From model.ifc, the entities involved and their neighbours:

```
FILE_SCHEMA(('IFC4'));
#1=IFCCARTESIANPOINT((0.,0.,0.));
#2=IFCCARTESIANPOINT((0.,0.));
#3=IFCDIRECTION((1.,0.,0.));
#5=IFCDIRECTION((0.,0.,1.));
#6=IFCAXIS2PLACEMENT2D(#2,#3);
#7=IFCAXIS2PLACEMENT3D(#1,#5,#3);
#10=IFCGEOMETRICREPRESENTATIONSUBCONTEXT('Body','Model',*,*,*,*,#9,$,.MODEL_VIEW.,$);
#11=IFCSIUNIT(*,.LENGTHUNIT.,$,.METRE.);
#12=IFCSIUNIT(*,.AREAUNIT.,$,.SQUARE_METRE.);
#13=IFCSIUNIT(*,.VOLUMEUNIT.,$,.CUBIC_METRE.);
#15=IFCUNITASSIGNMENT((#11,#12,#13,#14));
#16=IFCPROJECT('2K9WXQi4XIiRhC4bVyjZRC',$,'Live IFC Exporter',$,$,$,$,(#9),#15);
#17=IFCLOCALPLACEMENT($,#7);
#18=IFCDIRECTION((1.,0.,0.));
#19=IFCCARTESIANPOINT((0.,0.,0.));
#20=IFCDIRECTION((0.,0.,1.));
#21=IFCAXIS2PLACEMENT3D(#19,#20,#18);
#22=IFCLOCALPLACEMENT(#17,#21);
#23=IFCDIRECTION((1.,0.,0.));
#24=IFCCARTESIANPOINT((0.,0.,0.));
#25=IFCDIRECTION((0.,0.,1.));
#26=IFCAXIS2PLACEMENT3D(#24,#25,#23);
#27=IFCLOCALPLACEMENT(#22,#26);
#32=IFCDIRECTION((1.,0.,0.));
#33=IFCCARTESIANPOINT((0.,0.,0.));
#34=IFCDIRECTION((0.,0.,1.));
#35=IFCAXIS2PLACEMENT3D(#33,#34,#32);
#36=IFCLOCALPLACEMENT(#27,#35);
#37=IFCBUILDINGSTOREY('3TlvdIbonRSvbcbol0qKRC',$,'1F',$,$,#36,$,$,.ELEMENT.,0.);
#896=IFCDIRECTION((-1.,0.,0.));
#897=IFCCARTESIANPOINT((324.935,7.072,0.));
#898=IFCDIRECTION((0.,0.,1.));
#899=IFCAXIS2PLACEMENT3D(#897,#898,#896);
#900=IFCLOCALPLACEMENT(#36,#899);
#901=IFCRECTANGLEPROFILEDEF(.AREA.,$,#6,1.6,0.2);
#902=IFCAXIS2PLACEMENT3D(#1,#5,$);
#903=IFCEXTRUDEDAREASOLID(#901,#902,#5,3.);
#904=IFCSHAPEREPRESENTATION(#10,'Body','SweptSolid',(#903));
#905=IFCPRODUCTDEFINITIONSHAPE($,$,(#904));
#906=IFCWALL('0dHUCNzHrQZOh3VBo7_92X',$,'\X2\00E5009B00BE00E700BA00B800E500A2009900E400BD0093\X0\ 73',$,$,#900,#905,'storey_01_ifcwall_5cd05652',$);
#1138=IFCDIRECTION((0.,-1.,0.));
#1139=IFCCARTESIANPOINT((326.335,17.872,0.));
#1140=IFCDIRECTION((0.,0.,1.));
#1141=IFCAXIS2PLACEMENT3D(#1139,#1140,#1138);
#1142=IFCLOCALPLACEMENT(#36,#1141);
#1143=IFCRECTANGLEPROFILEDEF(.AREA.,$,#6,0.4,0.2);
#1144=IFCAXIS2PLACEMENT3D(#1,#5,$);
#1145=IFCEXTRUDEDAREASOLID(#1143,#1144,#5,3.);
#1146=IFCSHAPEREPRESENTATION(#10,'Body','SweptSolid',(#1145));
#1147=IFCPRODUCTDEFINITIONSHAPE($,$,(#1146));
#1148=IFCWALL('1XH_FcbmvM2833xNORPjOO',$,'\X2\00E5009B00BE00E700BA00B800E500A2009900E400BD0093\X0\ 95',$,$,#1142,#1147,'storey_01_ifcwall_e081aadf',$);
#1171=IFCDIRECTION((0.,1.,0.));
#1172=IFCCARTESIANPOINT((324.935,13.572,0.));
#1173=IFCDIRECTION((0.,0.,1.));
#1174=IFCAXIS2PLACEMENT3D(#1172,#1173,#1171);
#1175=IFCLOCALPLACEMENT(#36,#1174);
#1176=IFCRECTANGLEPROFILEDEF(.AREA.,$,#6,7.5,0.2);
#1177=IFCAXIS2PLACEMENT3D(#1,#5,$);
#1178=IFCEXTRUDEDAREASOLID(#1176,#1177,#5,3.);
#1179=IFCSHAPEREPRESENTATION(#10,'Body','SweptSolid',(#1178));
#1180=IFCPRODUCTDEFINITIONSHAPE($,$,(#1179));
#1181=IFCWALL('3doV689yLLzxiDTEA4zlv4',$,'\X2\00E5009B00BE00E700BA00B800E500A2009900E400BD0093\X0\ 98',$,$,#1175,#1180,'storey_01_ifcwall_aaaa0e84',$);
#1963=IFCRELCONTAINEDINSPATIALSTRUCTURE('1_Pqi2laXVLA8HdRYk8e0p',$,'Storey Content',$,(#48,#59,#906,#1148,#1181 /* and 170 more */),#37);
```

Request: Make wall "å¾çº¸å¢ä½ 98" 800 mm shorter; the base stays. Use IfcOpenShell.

```python
import ifcopenshell
import ifcopenshell.geom
import ifcopenshell.util.representation
import ifcopenshell.util.shape
import ifcopenshell.util.unit

model = ifcopenshell.open("model.ifc")
unit_scale = ifcopenshell.util.unit.calculate_unit_scale(model)
settings = ifcopenshell.geom.settings()


def volume(element):
    """Net volume in cubic metres, openings subtracted."""
    shape = ifcopenshell.geom.create_shape(settings, element)
    return ifcopenshell.util.shape.get_volume(shape.geometry)


wall = model.by_guid("3doV689yLLzxiDTEA4zlv4")
before = volume(wall)

body = ifcopenshell.util.representation.get_representation(wall, "Model", "Body")
solid = body.Items[0]
old_height = solid.Depth
solid.Depth -= 0.8 / unit_scale
after = volume(wall)

print(f"height {old_height:g} -> {solid.Depth:g}, volume {before:.3f} -> {after:.3f} m3")

model.write("model-out.ifc")
```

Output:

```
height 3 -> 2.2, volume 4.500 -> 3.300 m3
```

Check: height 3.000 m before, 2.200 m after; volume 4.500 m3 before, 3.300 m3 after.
